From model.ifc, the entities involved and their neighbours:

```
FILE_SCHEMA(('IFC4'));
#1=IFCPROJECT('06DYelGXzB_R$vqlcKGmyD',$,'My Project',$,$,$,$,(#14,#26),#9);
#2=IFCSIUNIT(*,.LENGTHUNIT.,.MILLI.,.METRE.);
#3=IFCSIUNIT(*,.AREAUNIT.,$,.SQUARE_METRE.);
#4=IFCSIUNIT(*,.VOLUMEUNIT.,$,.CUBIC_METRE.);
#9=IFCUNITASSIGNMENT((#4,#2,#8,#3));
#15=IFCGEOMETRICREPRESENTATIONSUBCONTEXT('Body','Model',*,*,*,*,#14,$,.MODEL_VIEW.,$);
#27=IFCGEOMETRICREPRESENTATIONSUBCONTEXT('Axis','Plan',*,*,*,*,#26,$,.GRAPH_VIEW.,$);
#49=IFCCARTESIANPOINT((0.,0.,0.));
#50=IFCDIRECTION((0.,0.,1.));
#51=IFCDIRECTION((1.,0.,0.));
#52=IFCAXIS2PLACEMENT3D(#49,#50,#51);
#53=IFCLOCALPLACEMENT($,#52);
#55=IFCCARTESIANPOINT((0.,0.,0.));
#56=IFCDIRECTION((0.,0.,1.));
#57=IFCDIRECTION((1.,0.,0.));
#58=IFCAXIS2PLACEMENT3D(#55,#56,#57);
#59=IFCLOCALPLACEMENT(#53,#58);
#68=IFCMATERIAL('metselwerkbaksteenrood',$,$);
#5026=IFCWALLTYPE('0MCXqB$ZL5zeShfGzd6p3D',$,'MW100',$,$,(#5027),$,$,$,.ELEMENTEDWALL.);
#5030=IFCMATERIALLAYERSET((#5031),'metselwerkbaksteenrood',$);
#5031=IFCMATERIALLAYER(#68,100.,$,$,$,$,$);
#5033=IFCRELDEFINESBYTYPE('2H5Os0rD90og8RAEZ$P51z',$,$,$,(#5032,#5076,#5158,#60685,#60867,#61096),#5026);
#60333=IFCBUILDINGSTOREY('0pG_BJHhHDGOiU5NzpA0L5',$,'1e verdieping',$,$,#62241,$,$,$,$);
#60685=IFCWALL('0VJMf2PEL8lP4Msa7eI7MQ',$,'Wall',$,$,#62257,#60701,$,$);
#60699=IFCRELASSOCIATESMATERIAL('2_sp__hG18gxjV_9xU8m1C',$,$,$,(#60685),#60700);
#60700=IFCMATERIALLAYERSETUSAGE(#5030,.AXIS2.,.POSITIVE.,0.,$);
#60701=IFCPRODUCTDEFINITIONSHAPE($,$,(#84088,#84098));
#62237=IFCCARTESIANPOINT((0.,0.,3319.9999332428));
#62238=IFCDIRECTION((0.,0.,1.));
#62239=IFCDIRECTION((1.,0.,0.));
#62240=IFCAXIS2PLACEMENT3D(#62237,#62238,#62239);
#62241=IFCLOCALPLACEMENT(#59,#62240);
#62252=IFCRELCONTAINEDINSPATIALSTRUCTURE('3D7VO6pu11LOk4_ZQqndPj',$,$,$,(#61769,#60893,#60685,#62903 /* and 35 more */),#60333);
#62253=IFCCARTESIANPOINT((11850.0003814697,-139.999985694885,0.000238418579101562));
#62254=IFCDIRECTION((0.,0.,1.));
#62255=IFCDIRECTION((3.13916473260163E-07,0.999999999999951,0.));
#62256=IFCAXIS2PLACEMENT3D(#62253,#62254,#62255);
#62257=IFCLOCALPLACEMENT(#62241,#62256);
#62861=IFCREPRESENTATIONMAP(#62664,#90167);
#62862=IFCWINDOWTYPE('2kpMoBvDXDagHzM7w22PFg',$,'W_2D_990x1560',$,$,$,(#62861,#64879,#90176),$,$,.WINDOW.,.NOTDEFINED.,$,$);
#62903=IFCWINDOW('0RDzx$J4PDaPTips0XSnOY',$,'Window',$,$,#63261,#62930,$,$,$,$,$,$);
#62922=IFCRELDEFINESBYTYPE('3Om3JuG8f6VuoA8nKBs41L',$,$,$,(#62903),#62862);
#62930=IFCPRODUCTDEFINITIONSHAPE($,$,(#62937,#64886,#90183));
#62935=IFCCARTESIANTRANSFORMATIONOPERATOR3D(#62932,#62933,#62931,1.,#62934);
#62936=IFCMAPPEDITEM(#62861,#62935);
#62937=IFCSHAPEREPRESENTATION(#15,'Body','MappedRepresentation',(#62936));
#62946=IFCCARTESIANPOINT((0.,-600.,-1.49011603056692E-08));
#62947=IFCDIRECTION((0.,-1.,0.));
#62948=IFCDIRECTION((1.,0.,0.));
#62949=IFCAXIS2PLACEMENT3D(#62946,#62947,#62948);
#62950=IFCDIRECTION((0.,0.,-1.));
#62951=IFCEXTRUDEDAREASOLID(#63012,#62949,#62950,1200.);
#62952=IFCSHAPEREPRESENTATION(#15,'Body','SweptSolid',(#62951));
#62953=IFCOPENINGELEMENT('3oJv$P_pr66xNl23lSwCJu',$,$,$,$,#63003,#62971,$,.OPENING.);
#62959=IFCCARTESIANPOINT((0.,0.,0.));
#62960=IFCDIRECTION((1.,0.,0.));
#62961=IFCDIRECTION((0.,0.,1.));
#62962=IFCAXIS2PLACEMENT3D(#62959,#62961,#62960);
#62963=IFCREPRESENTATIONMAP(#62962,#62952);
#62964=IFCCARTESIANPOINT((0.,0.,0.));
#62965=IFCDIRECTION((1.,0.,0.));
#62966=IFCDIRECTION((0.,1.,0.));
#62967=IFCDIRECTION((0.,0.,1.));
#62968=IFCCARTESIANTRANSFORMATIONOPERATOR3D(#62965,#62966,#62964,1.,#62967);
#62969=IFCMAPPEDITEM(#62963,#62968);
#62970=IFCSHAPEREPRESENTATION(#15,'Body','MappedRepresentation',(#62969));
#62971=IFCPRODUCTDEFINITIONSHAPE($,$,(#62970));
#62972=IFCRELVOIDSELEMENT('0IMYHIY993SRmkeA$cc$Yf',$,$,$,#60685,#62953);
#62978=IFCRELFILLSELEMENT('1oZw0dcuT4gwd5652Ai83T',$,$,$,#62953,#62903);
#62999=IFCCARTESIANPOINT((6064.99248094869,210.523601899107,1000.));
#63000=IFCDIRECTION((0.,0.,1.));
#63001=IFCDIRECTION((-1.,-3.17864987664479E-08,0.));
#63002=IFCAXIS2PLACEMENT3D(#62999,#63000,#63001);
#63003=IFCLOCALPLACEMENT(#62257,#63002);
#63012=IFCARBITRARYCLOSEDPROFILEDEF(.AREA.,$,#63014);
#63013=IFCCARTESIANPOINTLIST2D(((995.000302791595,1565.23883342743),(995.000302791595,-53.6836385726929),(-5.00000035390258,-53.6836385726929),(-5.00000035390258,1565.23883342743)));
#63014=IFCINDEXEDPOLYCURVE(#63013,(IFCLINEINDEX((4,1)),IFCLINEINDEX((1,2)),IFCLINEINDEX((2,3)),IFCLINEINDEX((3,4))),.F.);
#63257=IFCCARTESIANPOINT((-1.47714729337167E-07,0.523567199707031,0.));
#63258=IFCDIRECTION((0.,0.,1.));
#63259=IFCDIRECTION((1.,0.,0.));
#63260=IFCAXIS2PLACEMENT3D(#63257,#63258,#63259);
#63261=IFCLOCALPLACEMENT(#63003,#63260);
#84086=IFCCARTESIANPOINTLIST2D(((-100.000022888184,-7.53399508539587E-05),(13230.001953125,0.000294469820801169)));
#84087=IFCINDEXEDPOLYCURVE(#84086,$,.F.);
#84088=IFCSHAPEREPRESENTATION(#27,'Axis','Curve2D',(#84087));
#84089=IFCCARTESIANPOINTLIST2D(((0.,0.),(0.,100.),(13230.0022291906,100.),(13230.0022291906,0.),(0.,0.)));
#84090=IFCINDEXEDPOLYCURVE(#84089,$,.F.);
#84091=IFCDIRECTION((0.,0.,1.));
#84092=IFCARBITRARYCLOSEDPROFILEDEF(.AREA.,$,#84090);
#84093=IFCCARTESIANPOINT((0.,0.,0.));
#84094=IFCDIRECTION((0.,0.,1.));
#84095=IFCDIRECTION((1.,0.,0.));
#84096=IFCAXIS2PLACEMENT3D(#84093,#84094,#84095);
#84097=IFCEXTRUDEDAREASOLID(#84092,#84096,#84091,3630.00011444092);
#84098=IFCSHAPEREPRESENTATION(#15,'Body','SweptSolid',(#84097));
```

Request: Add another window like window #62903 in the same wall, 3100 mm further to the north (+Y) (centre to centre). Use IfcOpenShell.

```python
import ifcopenshell
import ifcopenshell.api.feature
import ifcopenshell.api.geometry
import ifcopenshell.api.root
import ifcopenshell.geom
import ifcopenshell.util.element
import ifcopenshell.util.placement
import ifcopenshell.util.shape

model = ifcopenshell.open("model.ifc")
settings = ifcopenshell.geom.settings()


def volume(element):
    """Net volume in cubic metres, openings subtracted."""
    shape = ifcopenshell.geom.create_shape(settings, element)
    return ifcopenshell.util.shape.get_volume(shape.geometry)


window = model.by_guid("0RDzx$J4PDaPTips0XSnOY")
opening = window.FillsVoids[0].RelatingOpeningElement
wall = opening.VoidsElements[0].RelatingBuildingElement
before = volume(wall)
shift = ifcopenshell.util.placement.get_local_placement(wall.ObjectPlacement)[:3, 0] * 3100.0

# copy_class copies the void relationship, type, container and properties, but no geometry.
new_opening = ifcopenshell.api.root.copy_class(model, product=opening)
new_opening.Representation = ifcopenshell.util.element.copy_deep(
    model, opening.Representation, exclude=["IfcGeometricRepresentationContext", "IfcRepresentationMap"]
)
new_window = ifcopenshell.api.root.copy_class(model, product=window)
new_window.Representation = ifcopenshell.util.element.copy_deep(
    model, window.Representation, exclude=["IfcGeometricRepresentationContext", "IfcRepresentationMap"]
)
ifcopenshell.api.feature.add_filling(model, opening=new_opening, element=new_window)

for old, new in ((opening, new_opening), (window, new_window)):
    matrix = ifcopenshell.util.placement.get_local_placement(old.ObjectPlacement)
    matrix[:3, 3] += shift
    ifcopenshell.api.geometry.edit_object_placement(model, product=new, matrix=matrix, is_si=False)

after = volume(wall)

print(f"wall volume {before:.3f} -> {after:.3f} m3")

model.write("model-out.ifc")
```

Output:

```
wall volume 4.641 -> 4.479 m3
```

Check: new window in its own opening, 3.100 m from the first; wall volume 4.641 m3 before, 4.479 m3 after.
